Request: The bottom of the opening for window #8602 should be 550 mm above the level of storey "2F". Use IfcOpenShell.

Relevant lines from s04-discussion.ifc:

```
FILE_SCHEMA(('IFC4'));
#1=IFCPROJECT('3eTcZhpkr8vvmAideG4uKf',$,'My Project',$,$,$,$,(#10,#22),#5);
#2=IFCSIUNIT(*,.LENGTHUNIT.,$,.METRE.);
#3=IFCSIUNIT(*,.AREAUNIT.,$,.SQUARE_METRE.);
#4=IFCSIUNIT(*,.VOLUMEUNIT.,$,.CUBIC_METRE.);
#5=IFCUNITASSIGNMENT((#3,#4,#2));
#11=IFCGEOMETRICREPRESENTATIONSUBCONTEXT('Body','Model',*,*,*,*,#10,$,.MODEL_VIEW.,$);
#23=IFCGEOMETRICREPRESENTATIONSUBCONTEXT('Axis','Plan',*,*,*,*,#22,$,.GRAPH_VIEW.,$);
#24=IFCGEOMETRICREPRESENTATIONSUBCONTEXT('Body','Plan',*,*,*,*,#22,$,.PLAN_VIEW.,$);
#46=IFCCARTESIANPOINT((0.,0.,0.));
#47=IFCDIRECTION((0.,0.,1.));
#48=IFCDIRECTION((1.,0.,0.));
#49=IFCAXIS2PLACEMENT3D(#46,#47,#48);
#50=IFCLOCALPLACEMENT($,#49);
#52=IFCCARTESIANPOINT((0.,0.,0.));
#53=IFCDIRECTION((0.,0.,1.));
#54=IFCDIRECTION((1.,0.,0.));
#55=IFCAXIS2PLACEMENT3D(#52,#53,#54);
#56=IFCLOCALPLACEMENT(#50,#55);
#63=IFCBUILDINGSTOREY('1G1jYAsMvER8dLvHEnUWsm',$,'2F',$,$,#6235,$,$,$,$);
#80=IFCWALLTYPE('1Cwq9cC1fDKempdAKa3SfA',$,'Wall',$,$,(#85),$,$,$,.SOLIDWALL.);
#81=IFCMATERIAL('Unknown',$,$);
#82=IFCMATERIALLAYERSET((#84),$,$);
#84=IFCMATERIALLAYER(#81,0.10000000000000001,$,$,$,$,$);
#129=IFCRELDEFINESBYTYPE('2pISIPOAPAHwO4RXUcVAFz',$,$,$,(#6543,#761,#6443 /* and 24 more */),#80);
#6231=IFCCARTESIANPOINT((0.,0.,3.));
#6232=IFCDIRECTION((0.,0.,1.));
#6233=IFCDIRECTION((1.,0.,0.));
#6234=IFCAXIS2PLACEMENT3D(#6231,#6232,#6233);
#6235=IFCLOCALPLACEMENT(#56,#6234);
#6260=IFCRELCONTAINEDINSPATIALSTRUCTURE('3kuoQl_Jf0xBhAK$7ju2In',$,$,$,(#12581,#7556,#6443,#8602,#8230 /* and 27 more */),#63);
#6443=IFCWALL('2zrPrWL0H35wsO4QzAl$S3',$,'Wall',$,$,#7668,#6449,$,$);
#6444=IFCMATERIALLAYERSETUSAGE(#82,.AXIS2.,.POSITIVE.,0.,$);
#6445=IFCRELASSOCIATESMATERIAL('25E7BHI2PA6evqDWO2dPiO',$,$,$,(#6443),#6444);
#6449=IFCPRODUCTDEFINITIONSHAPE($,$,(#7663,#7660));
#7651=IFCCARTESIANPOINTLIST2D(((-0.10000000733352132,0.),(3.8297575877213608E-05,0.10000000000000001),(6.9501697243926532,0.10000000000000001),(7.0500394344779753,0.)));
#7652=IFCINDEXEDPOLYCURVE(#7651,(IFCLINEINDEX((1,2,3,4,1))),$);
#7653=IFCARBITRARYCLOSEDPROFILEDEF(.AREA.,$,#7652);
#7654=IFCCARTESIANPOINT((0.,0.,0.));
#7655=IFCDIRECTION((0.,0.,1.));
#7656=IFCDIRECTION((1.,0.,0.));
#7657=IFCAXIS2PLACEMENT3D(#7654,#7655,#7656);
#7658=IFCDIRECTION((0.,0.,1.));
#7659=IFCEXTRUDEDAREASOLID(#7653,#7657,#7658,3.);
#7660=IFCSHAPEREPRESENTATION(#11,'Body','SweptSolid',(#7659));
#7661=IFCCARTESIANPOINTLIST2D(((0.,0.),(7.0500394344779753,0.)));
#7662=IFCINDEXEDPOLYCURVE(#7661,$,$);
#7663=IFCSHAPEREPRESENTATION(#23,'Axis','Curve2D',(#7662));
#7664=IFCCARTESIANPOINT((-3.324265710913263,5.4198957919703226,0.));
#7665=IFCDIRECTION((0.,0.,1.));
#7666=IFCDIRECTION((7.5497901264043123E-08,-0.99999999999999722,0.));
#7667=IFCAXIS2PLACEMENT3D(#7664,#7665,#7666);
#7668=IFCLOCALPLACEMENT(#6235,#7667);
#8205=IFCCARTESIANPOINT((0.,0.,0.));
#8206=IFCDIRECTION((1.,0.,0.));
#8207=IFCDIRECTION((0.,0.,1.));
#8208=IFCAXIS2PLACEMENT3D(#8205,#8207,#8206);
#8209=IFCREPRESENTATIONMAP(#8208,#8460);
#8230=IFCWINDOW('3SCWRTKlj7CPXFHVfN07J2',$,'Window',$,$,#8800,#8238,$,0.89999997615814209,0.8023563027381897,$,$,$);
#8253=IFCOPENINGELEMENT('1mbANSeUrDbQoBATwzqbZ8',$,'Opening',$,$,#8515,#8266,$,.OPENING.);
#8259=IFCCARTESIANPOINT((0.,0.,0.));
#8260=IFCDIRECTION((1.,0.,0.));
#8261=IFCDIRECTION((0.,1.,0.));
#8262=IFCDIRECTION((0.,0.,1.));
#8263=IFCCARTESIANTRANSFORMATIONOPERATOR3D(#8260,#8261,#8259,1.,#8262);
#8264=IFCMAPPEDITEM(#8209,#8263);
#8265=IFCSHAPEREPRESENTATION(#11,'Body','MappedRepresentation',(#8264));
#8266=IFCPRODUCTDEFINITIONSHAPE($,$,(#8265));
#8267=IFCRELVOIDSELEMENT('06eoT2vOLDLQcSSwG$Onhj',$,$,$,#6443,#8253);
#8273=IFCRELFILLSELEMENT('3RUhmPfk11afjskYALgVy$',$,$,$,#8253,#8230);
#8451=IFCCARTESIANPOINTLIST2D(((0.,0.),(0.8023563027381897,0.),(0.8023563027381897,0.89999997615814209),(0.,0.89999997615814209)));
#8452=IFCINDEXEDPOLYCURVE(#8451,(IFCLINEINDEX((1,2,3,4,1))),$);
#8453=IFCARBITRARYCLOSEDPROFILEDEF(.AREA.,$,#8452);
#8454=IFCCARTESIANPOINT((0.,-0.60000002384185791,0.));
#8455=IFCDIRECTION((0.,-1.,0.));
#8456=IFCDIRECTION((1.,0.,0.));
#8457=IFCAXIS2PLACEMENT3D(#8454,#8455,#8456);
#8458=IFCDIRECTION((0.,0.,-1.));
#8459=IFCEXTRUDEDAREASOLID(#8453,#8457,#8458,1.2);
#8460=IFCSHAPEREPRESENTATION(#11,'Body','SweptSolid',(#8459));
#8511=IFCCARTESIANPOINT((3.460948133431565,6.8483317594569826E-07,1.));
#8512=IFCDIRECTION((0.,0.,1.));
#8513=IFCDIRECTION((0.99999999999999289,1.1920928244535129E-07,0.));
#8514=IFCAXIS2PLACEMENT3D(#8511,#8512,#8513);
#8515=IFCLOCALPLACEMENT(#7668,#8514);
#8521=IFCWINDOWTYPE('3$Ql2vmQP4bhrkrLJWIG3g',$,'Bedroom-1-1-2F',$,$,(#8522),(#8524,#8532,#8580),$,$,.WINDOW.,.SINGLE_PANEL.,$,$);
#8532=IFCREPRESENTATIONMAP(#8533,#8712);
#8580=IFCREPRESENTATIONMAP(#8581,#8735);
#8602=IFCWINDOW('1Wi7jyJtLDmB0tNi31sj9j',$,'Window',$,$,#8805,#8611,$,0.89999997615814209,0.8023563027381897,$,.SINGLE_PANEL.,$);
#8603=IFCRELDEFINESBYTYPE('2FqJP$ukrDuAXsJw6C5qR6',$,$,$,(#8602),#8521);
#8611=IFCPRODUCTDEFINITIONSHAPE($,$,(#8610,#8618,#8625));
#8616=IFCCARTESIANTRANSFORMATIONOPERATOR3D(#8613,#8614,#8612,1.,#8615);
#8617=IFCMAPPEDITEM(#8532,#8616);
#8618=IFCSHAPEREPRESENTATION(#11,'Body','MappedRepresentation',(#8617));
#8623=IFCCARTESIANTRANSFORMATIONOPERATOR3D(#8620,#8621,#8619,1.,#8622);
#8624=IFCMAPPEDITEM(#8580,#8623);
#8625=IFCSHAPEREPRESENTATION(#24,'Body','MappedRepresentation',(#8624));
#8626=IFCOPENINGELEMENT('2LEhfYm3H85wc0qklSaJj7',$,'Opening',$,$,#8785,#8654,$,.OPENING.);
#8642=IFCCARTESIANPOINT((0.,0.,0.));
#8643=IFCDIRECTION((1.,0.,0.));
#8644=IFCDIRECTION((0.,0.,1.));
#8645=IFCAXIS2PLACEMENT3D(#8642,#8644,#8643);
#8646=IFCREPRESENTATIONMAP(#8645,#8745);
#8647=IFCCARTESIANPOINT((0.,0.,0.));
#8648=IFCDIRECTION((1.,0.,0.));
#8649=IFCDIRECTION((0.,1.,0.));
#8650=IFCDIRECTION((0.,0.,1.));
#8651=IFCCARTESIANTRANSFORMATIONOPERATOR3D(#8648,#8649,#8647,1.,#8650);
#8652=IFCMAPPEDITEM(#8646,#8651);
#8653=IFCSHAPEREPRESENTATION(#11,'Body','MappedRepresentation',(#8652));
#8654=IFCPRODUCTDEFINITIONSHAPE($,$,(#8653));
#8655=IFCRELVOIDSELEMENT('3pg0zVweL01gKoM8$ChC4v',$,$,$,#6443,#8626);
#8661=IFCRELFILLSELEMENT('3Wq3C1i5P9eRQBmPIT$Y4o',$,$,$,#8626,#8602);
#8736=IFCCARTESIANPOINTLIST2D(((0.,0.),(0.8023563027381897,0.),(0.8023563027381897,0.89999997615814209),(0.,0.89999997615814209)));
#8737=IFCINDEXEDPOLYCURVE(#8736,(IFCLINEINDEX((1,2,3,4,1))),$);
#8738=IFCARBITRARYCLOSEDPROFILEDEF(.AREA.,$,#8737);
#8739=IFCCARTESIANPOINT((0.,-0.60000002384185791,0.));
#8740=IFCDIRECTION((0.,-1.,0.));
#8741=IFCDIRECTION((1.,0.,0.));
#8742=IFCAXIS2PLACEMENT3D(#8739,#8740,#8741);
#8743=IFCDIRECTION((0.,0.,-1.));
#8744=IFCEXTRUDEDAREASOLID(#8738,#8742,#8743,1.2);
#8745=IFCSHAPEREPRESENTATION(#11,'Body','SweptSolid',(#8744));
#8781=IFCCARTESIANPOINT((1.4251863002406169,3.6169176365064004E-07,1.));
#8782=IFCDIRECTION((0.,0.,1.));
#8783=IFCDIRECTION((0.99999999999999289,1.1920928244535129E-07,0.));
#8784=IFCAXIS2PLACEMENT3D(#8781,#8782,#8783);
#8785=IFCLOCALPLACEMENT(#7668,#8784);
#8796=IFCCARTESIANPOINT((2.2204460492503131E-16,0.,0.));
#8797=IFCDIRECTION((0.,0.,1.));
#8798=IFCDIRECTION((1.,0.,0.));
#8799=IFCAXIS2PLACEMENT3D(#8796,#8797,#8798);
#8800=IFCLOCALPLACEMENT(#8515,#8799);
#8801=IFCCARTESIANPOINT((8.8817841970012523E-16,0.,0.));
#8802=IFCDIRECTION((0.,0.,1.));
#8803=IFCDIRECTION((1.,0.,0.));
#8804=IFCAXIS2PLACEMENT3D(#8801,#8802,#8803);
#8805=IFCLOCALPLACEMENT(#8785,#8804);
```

```python
import numpy as np
import ifcopenshell
import ifcopenshell.api.geometry
import ifcopenshell.geom
import ifcopenshell.util.element
import ifcopenshell.util.placement
import ifcopenshell.util.shape
import ifcopenshell.util.unit

model = ifcopenshell.open("s04-discussion.ifc")
unit_scale = ifcopenshell.util.unit.calculate_unit_scale(model)

window = model.by_guid("1Wi7jyJtLDmB0tNi31sj9j")
opening = window.FillsVoids[0].RelatingOpeningElement
storey = ifcopenshell.util.element.get_container(window, ifc_class="IfcBuildingStorey")
level = ifcopenshell.util.placement.get_local_placement(storey.ObjectPlacement)[2, 3]

# The opening's origin need not be at the sill, so measure its lowest point.
shape = ifcopenshell.geom.create_shape(ifcopenshell.geom.settings(), opening)
bottom = ifcopenshell.util.shape.get_shape_bottom_elevation(shape, shape.geometry) / unit_scale
dz = level + 0.55 / unit_scale - bottom

shift = np.array([0.0, 0.0, dz])
# The window is placed relative to its opening, so it follows when the opening moves.
matrix = ifcopenshell.util.placement.get_local_placement(opening.ObjectPlacement)
matrix[:3, 3] += shift
ifcopenshell.api.geometry.edit_object_placement(
    model, product=opening, matrix=matrix, is_si=False, should_transform_children=True
)

print(f"moved by {dz * unit_scale:+.3f} m")

model.write("s04-discussion_rev.ifc")
```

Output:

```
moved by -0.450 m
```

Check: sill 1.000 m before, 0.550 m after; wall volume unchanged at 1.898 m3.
